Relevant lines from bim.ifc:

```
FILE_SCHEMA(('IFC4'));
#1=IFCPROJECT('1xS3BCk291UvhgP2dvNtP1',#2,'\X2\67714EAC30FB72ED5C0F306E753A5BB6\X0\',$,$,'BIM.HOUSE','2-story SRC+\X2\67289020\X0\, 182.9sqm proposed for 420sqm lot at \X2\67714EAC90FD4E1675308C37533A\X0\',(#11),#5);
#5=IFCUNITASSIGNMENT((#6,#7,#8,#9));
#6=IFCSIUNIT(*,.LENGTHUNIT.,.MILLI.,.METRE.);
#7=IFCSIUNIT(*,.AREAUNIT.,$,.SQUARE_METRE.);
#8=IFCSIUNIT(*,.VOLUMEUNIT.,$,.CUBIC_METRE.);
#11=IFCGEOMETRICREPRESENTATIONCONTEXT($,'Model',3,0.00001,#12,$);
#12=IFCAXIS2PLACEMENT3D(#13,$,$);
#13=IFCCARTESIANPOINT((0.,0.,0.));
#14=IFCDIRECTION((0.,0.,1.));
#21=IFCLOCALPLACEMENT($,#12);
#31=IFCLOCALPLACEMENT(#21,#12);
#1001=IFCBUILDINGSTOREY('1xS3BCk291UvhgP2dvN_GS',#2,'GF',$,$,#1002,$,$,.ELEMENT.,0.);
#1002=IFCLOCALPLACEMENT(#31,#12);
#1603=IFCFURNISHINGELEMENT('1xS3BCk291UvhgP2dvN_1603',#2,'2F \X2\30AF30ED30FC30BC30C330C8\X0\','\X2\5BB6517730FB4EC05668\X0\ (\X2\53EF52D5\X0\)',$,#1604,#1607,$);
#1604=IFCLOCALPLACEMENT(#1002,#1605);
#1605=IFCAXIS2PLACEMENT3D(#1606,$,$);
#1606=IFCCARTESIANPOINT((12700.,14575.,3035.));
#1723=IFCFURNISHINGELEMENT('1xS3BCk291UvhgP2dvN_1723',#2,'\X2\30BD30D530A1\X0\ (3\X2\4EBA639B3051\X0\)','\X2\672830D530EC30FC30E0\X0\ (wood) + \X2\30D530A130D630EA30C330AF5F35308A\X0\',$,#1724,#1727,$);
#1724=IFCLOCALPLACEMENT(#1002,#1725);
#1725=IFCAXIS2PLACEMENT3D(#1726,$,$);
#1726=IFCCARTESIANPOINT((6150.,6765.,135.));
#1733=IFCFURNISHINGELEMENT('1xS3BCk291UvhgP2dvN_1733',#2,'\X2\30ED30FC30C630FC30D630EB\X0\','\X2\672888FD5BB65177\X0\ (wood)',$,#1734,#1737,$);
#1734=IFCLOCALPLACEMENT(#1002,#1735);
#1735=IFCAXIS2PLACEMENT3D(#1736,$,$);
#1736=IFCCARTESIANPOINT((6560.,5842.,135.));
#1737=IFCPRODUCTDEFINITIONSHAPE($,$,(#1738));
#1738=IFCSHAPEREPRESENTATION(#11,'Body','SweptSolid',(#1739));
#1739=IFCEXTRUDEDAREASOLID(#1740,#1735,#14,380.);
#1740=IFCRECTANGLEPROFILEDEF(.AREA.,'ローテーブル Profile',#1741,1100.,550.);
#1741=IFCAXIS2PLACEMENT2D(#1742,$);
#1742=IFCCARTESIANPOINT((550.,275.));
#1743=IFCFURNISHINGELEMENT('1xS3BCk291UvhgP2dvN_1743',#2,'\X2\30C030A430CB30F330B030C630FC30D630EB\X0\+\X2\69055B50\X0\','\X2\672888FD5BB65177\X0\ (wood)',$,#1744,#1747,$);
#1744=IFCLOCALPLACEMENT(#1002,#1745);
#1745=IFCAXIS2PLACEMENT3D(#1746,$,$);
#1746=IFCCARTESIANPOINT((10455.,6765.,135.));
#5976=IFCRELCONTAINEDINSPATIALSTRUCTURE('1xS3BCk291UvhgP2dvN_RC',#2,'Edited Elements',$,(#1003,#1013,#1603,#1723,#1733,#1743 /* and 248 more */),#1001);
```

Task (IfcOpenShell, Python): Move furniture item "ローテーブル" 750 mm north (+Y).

```python
import ifcopenshell
import ifcopenshell.api.geometry
import ifcopenshell.util.placement

model = ifcopenshell.open("bim.ifc")

item = model.by_guid("1xS3BCk291UvhgP2dvN_1733")
matrix = ifcopenshell.util.placement.get_local_placement(item.ObjectPlacement)
matrix[1, 3] += 750.0
ifcopenshell.api.geometry.edit_object_placement(model, product=item, matrix=matrix, is_si=False)

print(ifcopenshell.util.placement.get_local_placement(item.ObjectPlacement).round(3) + 0.0)

model.write("bim-out.ifc")
```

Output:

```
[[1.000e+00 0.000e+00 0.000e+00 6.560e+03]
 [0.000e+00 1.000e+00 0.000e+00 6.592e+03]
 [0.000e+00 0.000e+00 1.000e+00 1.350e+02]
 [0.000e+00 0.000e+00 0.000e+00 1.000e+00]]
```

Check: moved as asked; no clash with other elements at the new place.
